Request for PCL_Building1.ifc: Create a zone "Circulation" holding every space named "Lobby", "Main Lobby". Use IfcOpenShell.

First a look at what the model holds.

```python
import ifcopenshell

model = ifcopenshell.open("PCL_Building1.ifc")
print(model.schema)
seen = {}
for space in model.by_type("IfcSpace"):
    seen[space.LongName] = seen.get(space.LongName, 0) + 1
for name, count in sorted(seen.items(), key=str):
    print(count, "x", name)
print("zones:", [z.Name for z in model.by_type("IfcZone")][:20])
```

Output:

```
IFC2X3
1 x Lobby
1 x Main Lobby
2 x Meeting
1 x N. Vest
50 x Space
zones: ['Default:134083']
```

```python
import ifcopenshell
import ifcopenshell.api.group
import ifcopenshell.api.root

model = ifcopenshell.open("PCL_Building1.ifc")

names = {"Lobby", "Main Lobby"}
spaces = [s for s in model.by_type("IfcSpace") if s.LongName in names]

zone = ifcopenshell.api.root.create_entity(model, ifc_class="IfcZone", name="Circulation")
ifcopenshell.api.group.assign_group(model, products=spaces, group=zone)
print(len(spaces), "spaces in", zone.Name)

model.write("PCL_Building1_updated.ifc")
```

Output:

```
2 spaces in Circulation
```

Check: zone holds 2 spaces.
